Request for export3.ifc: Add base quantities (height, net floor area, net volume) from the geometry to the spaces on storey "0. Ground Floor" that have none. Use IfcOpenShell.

First a look at what the model holds.

```python
import ifcopenshell
import ifcopenshell.util.element
import ifcopenshell.util.unit

model = ifcopenshell.open("export3.ifc")
print(model.schema)
for unit_type in ("LENGTHUNIT", "AREAUNIT", "VOLUMEUNIT"):
    print(unit_type, ifcopenshell.util.unit.calculate_unit_scale(model, unit_type))
storey = next(s for s in model.by_type("IfcBuildingStorey") if s.Name == "0. Ground Floor")
spaces = [e for e in ifcopenshell.util.element.get_decomposition(storey) if e.is_a("IfcSpace")]
for e in sorted(spaces, key=lambda e: e.id()):
    print(e.id(), e.is_a(), e.Name, list(ifcopenshell.util.element.get_psets(e, qtos_only=True)), sep=" | ")
```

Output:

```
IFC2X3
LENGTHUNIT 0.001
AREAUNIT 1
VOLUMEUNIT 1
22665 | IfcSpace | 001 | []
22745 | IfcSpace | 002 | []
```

```python
import ifcopenshell
import ifcopenshell.api.pset
import ifcopenshell.geom
import ifcopenshell.util.element
import ifcopenshell.util.shape
import ifcopenshell.util.unit

model = ifcopenshell.open("export3.ifc")
unit_scale = ifcopenshell.util.unit.calculate_unit_scale(model)
area_scale = ifcopenshell.util.unit.calculate_unit_scale(model, "AREAUNIT")
volume_scale = ifcopenshell.util.unit.calculate_unit_scale(model, "VOLUMEUNIT")
settings = ifcopenshell.geom.settings()

storey = next(s for s in model.by_type("IfcBuildingStorey") if s.Name == "0. Ground Floor")
spaces = [e for e in ifcopenshell.util.element.get_decomposition(storey) if e.is_a("IfcSpace")]

for e in sorted(spaces, key=lambda e: e.id()):
    if ifcopenshell.util.element.get_psets(e, qtos_only=True, should_inherit=False):
        continue
    # Geometry comes back in metres, in the element's own axes.
    shape = ifcopenshell.geom.create_shape(settings, e)
    values = {
        "Height": ifcopenshell.util.shape.get_z(shape.geometry) / unit_scale,
        "NetFloorArea": ifcopenshell.util.shape.get_footprint_area(shape.geometry) / area_scale,
        "NetVolume": ifcopenshell.util.shape.get_volume(shape.geometry) / volume_scale,
    }
    qto = ifcopenshell.api.pset.add_qto(model, product=e, name="BaseQuantities")
    ifcopenshell.api.pset.edit_qto(model, qto=qto, properties=values)
    print(e.id(), {k: round(v, 3) for k, v in values.items()})

model.write("export3-out.ifc")
```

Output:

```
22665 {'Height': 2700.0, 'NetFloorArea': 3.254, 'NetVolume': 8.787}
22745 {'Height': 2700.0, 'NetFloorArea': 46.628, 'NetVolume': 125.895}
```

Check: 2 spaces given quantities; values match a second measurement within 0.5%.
